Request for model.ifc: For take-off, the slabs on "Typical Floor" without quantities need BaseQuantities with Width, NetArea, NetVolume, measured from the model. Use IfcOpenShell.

First a look at what the model holds.

```python
import ifcopenshell
import ifcopenshell.util.element
import ifcopenshell.util.unit

model = ifcopenshell.open("model.ifc")
print(model.schema)
for unit_type in ("LENGTHUNIT", "AREAUNIT", "VOLUMEUNIT"):
    print(unit_type, ifcopenshell.util.unit.calculate_unit_scale(model, unit_type))
storey = next(s for s in model.by_type("IfcBuildingStorey") if s.Name == "Typical Floor")
slabs = [e for e in ifcopenshell.util.element.get_decomposition(storey) if e.is_a("IfcSlab")]
for e in sorted(slabs, key=lambda e: e.id()):
    print(e.id(), e.is_a(), e.Name, list(ifcopenshell.util.element.get_psets(e, qtos_only=True)), sep=" | ")
```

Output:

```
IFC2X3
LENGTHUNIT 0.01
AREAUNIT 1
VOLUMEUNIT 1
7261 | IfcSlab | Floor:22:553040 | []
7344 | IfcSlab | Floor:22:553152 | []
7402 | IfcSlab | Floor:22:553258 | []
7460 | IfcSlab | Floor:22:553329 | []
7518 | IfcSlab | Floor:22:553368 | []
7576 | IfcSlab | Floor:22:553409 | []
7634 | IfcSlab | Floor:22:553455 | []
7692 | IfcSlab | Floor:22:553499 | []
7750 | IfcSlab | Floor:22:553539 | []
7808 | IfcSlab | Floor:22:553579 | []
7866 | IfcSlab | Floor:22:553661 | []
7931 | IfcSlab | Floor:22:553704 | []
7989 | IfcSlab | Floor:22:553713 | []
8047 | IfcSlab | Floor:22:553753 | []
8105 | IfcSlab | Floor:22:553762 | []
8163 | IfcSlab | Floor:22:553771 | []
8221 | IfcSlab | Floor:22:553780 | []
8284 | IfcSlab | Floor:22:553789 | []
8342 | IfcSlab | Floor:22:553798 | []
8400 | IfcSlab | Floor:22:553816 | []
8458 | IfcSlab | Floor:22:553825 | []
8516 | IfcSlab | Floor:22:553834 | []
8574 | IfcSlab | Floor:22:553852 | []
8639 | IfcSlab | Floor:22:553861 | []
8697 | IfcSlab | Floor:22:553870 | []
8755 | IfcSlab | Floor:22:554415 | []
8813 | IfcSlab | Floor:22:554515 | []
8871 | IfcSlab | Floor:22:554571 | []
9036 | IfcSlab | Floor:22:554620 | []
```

```python
import ifcopenshell
import ifcopenshell.api.pset
import ifcopenshell.geom
import ifcopenshell.util.element
import ifcopenshell.util.shape
import ifcopenshell.util.unit

model = ifcopenshell.open("model.ifc")
unit_scale = ifcopenshell.util.unit.calculate_unit_scale(model)
area_scale = ifcopenshell.util.unit.calculate_unit_scale(model, "AREAUNIT")
volume_scale = ifcopenshell.util.unit.calculate_unit_scale(model, "VOLUMEUNIT")
settings = ifcopenshell.geom.settings()

storey = next(s for s in model.by_type("IfcBuildingStorey") if s.Name == "Typical Floor")
slabs = [e for e in ifcopenshell.util.element.get_decomposition(storey) if e.is_a("IfcSlab")]

for e in sorted(slabs, key=lambda e: e.id()):
    if ifcopenshell.util.element.get_psets(e, qtos_only=True, should_inherit=False):
        continue
    # Geometry comes back in metres, in the element's own axes.
    shape = ifcopenshell.geom.create_shape(settings, e)
    values = {
        "Width": ifcopenshell.util.shape.get_z(shape.geometry) / unit_scale,
        "NetArea": ifcopenshell.util.shape.get_footprint_area(shape.geometry) / area_scale,
        "NetVolume": ifcopenshell.util.shape.get_volume(shape.geometry) / volume_scale,
    }
    qto = ifcopenshell.api.pset.add_qto(model, product=e, name="BaseQuantities")
    ifcopenshell.api.pset.edit_qto(model, qto=qto, properties=values)
    print(e.id(), {k: round(v, 3) for k, v in values.items()})

model.write("model_updated.ifc")
```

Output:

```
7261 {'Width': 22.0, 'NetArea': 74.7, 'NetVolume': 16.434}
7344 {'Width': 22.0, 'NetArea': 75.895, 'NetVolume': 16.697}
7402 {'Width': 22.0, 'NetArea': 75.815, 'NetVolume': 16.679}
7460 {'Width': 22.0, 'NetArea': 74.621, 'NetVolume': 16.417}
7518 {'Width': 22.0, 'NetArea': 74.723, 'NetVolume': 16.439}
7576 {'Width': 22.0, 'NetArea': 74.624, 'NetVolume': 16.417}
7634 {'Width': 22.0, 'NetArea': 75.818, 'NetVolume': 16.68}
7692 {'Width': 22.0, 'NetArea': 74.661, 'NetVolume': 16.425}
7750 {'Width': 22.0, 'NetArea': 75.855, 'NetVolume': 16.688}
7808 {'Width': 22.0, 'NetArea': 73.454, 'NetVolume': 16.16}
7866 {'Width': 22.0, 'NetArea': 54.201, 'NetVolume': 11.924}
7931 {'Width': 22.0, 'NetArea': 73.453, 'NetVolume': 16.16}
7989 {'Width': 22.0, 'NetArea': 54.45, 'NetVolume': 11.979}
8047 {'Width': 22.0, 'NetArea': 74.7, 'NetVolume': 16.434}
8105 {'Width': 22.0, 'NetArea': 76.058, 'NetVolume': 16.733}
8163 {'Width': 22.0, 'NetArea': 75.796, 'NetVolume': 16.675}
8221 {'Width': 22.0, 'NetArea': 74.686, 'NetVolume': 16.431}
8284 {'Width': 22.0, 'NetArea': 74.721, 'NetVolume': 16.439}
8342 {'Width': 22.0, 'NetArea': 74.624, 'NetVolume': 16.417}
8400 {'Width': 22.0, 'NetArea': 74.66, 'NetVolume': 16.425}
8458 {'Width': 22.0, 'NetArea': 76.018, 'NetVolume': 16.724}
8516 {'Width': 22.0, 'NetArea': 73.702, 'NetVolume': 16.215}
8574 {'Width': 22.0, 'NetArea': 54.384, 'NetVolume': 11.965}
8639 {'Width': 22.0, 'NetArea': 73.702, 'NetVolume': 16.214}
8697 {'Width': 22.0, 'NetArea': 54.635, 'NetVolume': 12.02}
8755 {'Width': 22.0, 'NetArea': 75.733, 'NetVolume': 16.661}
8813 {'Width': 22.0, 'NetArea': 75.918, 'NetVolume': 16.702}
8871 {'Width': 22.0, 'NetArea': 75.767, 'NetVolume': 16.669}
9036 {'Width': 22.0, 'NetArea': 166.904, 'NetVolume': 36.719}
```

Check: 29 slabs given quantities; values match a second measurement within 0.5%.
